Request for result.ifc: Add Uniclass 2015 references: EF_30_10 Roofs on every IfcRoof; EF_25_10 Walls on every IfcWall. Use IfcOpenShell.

First a look at what the model holds.

```python
import ifcopenshell

model = ifcopenshell.open("result.ifc")
print(model.schema)
print("classifications:", [c.Name for c in model.by_type("IfcClassification")])
for ifc_class in ("IfcDoor", "IfcRoof", "IfcStair", "IfcWall", "IfcWindow"):
    print(ifc_class, len(model.by_type(ifc_class)))
```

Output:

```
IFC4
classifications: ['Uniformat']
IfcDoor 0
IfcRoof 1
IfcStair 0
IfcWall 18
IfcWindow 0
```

```python
import ifcopenshell
import ifcopenshell.api.classification

model = ifcopenshell.open("result.ifc")

system = ifcopenshell.api.classification.add_classification(model, classification="Uniclass 2015")

codes = {
    "IfcRoof": ("EF_30_10", "Roofs"),
    "IfcWall": ("EF_25_10", "Walls"),
}
for ifc_class, (code, name) in codes.items():
    products = model.by_type(ifc_class)
    ifcopenshell.api.classification.add_reference(
        model, products=products, classification=system, identification=code, name=name
    )
    print(code, len(products))

model.write("result_updated.ifc")
```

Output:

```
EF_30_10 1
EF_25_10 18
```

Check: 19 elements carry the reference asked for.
